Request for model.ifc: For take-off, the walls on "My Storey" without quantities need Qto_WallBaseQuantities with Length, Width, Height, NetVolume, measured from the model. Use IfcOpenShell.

First a look at what the model holds.

```python
import ifcopenshell
import ifcopenshell.util.element
import ifcopenshell.util.unit

model = ifcopenshell.open("model.ifc")
print(model.schema)
for unit_type in ("LENGTHUNIT", "AREAUNIT", "VOLUMEUNIT"):
    print(unit_type, ifcopenshell.util.unit.calculate_unit_scale(model, unit_type))
storey = next(s for s in model.by_type("IfcBuildingStorey") if s.Name == "My Storey")
walls = [e for e in ifcopenshell.util.element.get_decomposition(storey) if e.is_a("IfcWall")]
for e in sorted(walls, key=lambda e: e.id()):
    print(e.id(), e.is_a(), e.Name, list(ifcopenshell.util.element.get_psets(e, qtos_only=True)), sep=" | ")
```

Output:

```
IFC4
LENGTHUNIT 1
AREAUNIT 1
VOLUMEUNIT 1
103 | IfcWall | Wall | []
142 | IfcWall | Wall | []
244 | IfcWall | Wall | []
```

```python
import ifcopenshell
import ifcopenshell.api.pset
import ifcopenshell.geom
import ifcopenshell.util.element
import ifcopenshell.util.shape
import ifcopenshell.util.unit

model = ifcopenshell.open("model.ifc")
unit_scale = ifcopenshell.util.unit.calculate_unit_scale(model)
volume_scale = ifcopenshell.util.unit.calculate_unit_scale(model, "VOLUMEUNIT")
settings = ifcopenshell.geom.settings()

storey = next(s for s in model.by_type("IfcBuildingStorey") if s.Name == "My Storey")
walls = [e for e in ifcopenshell.util.element.get_decomposition(storey) if e.is_a("IfcWall")]

for e in sorted(walls, key=lambda e: e.id()):
    if ifcopenshell.util.element.get_psets(e, qtos_only=True, should_inherit=False):
        continue
    # Geometry comes back in metres, in the element's own axes.
    shape = ifcopenshell.geom.create_shape(settings, e)
    values = {
        "Length": ifcopenshell.util.shape.get_x(shape.geometry) / unit_scale,
        "Width": ifcopenshell.util.shape.get_y(shape.geometry) / unit_scale,
        "Height": ifcopenshell.util.shape.get_z(shape.geometry) / unit_scale,
        "NetVolume": ifcopenshell.util.shape.get_volume(shape.geometry) / volume_scale,
    }
    qto = ifcopenshell.api.pset.add_qto(model, product=e, name="Qto_WallBaseQuantities")
    ifcopenshell.api.pset.edit_qto(model, qto=qto, properties=values)
    print(e.id(), {k: round(v, 3) for k, v in values.items()})

model.write("model-out.ifc")
```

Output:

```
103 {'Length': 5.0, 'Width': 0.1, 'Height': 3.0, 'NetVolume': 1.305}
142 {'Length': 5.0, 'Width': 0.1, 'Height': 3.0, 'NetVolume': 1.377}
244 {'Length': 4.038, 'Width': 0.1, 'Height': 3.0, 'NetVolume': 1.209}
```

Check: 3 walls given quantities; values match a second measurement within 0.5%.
